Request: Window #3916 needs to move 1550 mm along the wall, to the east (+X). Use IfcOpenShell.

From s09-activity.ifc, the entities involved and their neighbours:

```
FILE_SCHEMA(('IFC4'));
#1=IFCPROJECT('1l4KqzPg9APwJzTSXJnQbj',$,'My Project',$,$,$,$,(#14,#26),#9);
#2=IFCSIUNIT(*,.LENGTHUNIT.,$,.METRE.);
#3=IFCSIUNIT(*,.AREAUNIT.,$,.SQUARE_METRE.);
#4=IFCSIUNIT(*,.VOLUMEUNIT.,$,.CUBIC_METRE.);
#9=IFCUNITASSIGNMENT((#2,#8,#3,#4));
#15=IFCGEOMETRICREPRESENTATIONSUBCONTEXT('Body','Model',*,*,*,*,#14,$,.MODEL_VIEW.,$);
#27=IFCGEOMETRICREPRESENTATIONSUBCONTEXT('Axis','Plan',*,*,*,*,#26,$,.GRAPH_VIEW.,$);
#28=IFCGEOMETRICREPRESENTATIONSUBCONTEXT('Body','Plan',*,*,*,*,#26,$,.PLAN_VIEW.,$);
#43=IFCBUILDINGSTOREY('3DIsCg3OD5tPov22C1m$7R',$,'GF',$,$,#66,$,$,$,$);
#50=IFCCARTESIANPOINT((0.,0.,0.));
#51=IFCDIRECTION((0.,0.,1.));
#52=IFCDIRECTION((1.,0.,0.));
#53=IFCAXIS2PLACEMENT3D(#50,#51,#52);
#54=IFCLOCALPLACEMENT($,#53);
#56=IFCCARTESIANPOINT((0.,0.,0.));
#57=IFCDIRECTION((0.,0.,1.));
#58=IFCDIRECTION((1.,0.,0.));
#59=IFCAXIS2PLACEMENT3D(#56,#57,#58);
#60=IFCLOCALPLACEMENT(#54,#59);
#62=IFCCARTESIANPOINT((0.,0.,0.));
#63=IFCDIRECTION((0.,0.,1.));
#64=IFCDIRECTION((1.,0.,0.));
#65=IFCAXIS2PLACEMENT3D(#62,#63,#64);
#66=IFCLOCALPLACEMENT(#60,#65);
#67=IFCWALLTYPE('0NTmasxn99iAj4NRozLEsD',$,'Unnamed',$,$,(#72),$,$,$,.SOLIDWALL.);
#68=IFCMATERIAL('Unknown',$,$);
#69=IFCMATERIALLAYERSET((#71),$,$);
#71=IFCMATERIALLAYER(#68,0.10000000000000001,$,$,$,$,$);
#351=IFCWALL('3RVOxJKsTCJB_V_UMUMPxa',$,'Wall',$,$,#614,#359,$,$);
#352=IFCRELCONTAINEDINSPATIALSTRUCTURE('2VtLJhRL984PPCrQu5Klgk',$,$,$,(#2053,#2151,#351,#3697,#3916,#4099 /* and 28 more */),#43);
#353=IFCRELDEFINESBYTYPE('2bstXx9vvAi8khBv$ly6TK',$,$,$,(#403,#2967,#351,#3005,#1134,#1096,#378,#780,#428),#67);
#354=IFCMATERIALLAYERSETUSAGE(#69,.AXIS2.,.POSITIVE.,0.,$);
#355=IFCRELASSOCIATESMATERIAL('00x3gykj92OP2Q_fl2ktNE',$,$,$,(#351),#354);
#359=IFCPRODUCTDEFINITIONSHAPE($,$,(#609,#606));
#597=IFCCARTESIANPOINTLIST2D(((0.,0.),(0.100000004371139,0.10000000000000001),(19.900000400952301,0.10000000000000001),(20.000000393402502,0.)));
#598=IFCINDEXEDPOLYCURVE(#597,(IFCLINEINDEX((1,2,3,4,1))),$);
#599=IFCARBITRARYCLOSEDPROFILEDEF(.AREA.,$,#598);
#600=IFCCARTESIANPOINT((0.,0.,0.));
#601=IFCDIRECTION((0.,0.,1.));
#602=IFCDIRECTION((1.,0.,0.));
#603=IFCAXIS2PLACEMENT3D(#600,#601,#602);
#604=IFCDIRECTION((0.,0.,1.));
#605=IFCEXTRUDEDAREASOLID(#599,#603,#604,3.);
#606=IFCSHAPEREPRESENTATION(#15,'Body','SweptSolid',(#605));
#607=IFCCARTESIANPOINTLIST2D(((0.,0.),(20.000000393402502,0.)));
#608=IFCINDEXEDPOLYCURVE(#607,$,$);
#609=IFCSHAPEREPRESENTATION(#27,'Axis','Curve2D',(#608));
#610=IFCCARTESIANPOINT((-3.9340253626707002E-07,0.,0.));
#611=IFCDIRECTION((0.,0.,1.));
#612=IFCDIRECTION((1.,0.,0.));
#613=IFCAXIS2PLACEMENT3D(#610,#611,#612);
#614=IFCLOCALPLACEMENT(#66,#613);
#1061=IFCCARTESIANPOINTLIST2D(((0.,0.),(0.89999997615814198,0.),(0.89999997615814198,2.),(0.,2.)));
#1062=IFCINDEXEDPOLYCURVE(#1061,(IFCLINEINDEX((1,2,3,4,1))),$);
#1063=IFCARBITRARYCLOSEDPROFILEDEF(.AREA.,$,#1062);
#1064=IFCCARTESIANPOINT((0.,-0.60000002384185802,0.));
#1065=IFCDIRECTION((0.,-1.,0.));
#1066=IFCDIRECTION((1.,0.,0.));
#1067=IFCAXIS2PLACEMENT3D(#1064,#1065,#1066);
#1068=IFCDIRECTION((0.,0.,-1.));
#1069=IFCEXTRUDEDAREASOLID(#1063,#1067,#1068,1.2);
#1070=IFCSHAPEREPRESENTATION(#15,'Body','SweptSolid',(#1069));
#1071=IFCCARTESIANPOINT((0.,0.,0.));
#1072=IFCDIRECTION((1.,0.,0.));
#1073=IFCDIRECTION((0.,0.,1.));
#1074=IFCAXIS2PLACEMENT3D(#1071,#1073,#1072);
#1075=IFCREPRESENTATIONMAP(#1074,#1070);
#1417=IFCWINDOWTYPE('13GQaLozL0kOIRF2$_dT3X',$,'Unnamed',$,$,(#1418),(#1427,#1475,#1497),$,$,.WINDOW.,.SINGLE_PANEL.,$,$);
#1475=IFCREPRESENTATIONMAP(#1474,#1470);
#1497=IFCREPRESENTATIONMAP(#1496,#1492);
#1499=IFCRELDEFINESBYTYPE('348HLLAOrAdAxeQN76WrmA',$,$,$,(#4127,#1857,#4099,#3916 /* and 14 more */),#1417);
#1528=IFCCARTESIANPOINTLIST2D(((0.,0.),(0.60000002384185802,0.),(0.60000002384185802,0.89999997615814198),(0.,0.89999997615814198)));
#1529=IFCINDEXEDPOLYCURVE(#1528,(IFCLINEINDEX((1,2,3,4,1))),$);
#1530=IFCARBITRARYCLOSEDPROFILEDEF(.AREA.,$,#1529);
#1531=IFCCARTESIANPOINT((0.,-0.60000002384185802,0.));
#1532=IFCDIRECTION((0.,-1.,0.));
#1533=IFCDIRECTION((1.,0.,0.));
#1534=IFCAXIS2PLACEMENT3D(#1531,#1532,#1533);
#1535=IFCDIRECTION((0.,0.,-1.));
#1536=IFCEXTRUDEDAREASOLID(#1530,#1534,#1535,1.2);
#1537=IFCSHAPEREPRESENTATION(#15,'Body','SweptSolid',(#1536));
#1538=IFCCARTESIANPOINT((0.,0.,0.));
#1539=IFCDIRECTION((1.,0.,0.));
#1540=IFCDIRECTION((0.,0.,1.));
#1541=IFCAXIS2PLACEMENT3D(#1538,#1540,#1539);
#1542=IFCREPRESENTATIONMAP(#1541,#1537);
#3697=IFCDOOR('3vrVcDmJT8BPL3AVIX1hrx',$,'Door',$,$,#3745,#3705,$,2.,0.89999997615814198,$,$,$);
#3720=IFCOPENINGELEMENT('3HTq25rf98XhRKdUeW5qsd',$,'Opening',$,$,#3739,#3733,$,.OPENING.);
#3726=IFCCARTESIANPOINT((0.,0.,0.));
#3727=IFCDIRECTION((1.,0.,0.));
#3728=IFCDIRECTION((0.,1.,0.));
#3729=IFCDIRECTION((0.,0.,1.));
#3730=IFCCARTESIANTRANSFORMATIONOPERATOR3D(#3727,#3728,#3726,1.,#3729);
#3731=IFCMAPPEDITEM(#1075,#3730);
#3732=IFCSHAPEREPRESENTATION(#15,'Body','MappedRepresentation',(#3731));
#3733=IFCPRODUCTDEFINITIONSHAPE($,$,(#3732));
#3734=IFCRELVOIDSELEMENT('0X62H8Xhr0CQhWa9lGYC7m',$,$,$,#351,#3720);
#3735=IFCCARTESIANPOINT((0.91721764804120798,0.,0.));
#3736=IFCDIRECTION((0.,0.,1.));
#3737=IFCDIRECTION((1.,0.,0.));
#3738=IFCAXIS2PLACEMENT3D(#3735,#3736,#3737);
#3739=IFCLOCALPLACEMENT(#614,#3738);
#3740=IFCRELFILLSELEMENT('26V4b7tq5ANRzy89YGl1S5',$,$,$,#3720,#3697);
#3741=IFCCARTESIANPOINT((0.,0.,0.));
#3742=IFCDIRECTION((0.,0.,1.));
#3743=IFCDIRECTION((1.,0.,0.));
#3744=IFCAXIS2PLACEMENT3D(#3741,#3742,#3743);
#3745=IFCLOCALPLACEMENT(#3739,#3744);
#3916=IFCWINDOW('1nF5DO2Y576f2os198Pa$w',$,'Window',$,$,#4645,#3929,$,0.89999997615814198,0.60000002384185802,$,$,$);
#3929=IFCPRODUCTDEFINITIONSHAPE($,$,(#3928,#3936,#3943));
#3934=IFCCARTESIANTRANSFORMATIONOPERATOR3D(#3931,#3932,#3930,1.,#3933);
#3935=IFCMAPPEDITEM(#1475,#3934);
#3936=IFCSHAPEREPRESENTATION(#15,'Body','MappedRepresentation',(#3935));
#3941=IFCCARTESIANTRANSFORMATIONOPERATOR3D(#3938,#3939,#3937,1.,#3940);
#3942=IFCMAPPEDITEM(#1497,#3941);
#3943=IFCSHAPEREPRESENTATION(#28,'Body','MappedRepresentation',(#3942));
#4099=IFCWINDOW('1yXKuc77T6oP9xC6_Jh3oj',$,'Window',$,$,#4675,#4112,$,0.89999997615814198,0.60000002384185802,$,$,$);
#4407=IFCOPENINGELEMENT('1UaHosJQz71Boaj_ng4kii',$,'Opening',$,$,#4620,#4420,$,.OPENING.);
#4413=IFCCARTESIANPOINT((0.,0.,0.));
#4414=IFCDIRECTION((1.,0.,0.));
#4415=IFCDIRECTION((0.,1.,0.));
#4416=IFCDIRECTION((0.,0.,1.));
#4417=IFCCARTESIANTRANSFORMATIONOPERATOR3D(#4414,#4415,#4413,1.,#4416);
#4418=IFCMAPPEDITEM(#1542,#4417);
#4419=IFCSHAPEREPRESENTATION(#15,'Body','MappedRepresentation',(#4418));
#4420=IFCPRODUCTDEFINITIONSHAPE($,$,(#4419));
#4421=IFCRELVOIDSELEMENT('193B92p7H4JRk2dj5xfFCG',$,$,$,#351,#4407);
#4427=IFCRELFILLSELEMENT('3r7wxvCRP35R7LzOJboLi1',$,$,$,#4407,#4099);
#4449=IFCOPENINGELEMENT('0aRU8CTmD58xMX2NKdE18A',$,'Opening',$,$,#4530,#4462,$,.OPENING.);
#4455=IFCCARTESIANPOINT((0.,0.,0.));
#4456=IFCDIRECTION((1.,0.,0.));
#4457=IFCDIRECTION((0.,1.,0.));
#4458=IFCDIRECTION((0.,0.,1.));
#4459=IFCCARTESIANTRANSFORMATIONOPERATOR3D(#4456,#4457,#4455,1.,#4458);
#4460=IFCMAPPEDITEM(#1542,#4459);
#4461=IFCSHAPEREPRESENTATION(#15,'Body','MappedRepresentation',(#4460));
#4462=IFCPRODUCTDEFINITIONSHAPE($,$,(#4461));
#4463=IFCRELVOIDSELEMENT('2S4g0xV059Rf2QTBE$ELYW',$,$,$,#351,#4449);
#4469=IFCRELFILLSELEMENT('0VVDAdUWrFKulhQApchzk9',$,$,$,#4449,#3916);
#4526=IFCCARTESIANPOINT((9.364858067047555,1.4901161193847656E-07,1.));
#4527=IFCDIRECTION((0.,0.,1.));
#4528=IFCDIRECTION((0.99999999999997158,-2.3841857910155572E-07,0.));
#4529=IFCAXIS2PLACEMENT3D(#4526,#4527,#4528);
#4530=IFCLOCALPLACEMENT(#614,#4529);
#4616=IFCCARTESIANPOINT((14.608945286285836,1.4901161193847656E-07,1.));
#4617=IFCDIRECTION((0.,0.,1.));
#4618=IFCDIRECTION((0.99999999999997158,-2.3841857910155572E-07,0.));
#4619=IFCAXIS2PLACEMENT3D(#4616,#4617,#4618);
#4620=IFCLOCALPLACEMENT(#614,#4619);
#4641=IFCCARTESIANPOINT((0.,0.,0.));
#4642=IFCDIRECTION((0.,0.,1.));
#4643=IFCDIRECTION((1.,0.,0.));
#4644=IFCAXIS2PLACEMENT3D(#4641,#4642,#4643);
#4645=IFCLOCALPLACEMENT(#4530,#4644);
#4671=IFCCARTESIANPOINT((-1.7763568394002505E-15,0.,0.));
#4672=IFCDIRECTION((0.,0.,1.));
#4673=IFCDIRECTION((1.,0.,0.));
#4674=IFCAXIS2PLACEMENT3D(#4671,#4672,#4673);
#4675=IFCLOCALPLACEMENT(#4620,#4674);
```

```python
import ifcopenshell
import ifcopenshell.api.geometry
import ifcopenshell.util.placement

model = ifcopenshell.open("s09-activity.ifc")

window = model.by_guid("1nF5DO2Y576f2os198Pa$w")
opening = window.FillsVoids[0].RelatingOpeningElement
wall = opening.VoidsElements[0].RelatingBuildingElement

wall_matrix = ifcopenshell.util.placement.get_local_placement(wall.ObjectPlacement)
shift = wall_matrix[:3, 0] * 1.55
before = ifcopenshell.util.placement.get_local_placement(window.ObjectPlacement)[:3, 3].copy()

# The window is placed relative to its opening, so it follows when the opening moves.
matrix = ifcopenshell.util.placement.get_local_placement(opening.ObjectPlacement)
matrix[:3, 3] += shift
ifcopenshell.api.geometry.edit_object_placement(
    model, product=opening, matrix=matrix, is_si=False, should_transform_children=True
)

after = ifcopenshell.util.placement.get_local_placement(window.ObjectPlacement)[:3, 3]
print("window moved by", (after - before).round(3) + 0.0)

model.write("s09-activity_edited.ifc")
```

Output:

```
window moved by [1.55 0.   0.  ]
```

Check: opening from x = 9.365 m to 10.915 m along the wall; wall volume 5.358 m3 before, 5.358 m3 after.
